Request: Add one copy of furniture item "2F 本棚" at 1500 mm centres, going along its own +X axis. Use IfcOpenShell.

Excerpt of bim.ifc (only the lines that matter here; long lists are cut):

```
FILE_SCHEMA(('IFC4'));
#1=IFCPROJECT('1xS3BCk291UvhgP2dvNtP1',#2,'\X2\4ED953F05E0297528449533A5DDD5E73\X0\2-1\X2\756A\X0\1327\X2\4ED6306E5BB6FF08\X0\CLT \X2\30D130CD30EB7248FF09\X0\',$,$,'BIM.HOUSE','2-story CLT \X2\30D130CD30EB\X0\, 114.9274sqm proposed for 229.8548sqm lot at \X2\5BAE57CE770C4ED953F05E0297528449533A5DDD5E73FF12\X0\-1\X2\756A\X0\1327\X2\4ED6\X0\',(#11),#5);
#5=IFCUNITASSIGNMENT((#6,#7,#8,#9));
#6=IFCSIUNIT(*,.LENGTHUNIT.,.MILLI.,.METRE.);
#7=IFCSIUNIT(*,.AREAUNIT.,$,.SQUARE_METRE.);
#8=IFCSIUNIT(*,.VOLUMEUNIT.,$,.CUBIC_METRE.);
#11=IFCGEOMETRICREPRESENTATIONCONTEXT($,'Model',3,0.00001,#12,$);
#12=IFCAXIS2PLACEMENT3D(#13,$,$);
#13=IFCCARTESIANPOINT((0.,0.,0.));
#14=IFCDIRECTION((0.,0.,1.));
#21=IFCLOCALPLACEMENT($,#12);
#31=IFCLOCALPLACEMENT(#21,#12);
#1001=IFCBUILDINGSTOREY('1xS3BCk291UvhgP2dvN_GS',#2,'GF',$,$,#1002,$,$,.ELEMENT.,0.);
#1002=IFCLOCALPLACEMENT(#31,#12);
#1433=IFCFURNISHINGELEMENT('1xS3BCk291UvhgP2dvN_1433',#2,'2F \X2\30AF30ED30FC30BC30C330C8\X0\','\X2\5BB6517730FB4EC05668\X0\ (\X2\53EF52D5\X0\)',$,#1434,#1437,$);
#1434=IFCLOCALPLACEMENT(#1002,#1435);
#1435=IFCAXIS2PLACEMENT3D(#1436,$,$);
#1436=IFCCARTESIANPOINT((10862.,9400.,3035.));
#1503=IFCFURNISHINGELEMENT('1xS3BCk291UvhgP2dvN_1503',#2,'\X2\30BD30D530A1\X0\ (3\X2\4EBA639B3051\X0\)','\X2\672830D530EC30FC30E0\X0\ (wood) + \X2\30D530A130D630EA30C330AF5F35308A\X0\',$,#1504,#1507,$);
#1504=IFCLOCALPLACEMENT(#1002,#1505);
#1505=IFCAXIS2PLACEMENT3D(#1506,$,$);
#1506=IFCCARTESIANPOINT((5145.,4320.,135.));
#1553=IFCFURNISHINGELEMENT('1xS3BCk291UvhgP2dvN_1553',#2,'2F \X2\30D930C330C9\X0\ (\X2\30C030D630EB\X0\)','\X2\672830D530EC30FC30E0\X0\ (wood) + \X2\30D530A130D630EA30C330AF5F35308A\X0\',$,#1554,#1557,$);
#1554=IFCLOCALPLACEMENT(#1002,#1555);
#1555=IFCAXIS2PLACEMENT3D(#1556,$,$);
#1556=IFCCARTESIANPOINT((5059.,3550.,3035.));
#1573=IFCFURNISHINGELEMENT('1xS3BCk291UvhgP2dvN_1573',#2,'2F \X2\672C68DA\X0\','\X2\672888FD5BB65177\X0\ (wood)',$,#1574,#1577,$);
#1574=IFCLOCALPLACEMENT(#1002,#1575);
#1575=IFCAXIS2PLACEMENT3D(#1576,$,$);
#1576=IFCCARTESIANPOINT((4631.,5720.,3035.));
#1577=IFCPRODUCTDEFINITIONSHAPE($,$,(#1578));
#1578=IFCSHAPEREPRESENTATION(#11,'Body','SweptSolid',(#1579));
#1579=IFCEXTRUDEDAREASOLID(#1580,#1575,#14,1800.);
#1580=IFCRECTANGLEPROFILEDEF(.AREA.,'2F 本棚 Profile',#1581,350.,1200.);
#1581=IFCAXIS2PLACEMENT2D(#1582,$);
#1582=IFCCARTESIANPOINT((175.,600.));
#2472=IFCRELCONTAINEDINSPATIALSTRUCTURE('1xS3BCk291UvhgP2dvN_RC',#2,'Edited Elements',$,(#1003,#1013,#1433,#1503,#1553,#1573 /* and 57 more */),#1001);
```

```python
import ifcopenshell
import ifcopenshell.api.geometry
import ifcopenshell.api.root
import ifcopenshell.util.element
import ifcopenshell.util.placement

model = ifcopenshell.open("bim.ifc")


def reuse_history(source, copy):
    """copy_class also copies each property set's owner history, people and application; keep the originals."""
    for rel in copy.IsDefinedBy:
        if rel.is_a("IfcRelDefinesByProperties") and (history := rel.RelatingPropertyDefinition.OwnerHistory):
            rel.RelatingPropertyDefinition.OwnerHistory = source.OwnerHistory
            ifcopenshell.util.element.remove_deep2(model, history)


source = model.by_guid("1xS3BCk291UvhgP2dvN_1573")
base = ifcopenshell.util.placement.get_local_placement(source.ObjectPlacement)
step = base[:3, 0] * 1500.0

for i in range(1, 2):
    copy = ifcopenshell.api.root.copy_class(model, product=source)
    copy.Representation = ifcopenshell.util.element.copy_deep(
        model, source.Representation, exclude=["IfcGeometricRepresentationContext", "IfcRepresentationMap"]
    )
    reuse_history(source, copy)
    matrix = base.copy()
    matrix[:3, 3] += i * step
    print("added at", matrix[:3, 3].round(3) + 0.0)
    ifcopenshell.api.geometry.edit_object_placement(model, product=copy, matrix=matrix, is_si=False)

model.write("bim_v2.ifc")
```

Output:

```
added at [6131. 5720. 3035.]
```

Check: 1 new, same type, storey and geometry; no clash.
